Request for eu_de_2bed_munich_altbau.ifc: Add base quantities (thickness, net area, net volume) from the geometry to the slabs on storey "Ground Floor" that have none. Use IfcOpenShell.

First a look at what the model holds.

```python
import ifcopenshell
import ifcopenshell.util.element
import ifcopenshell.util.unit

model = ifcopenshell.open("eu_de_2bed_munich_altbau.ifc")
print(model.schema)
for unit_type in ("LENGTHUNIT", "AREAUNIT", "VOLUMEUNIT"):
    print(unit_type, ifcopenshell.util.unit.calculate_unit_scale(model, unit_type))
storey = next(s for s in model.by_type("IfcBuildingStorey") if s.Name == "Ground Floor")
slabs = [e for e in ifcopenshell.util.element.get_decomposition(storey) if e.is_a("IfcSlab")]
for e in sorted(slabs, key=lambda e: e.id()):
    print(e.id(), e.is_a(), e.Name, list(ifcopenshell.util.element.get_psets(e, qtos_only=True)), sep=" | ")
```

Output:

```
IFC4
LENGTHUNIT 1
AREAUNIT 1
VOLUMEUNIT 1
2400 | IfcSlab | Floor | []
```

```python
import ifcopenshell
import ifcopenshell.api.pset
import ifcopenshell.geom
import ifcopenshell.util.element
import ifcopenshell.util.shape
import ifcopenshell.util.unit

model = ifcopenshell.open("eu_de_2bed_munich_altbau.ifc")
unit_scale = ifcopenshell.util.unit.calculate_unit_scale(model)
area_scale = ifcopenshell.util.unit.calculate_unit_scale(model, "AREAUNIT")
volume_scale = ifcopenshell.util.unit.calculate_unit_scale(model, "VOLUMEUNIT")
settings = ifcopenshell.geom.settings()

storey = next(s for s in model.by_type("IfcBuildingStorey") if s.Name == "Ground Floor")
slabs = [e for e in ifcopenshell.util.element.get_decomposition(storey) if e.is_a("IfcSlab")]

for e in sorted(slabs, key=lambda e: e.id()):
    if ifcopenshell.util.element.get_psets(e, qtos_only=True, should_inherit=False):
        continue
    # Geometry comes back in metres, in the element's own axes.
    shape = ifcopenshell.geom.create_shape(settings, e)
    values = {
        "Width": ifcopenshell.util.shape.get_z(shape.geometry) / unit_scale,
        "NetArea": ifcopenshell.util.shape.get_footprint_area(shape.geometry) / area_scale,
        "NetVolume": ifcopenshell.util.shape.get_volume(shape.geometry) / volume_scale,
    }
    qto = ifcopenshell.api.pset.add_qto(model, product=e, name="Qto_SlabBaseQuantities")
    ifcopenshell.api.pset.edit_qto(model, qto=qto, properties=values)
    print(e.id(), {k: round(v, 3) for k, v in values.items()})

model.write("eu_de_2bed_munich_altbau_updated.ifc")
```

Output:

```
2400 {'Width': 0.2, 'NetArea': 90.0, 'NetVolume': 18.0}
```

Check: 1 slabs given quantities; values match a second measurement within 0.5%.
